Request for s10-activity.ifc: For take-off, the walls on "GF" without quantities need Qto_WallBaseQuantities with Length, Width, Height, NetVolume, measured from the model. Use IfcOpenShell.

First a look at what the model holds.

```python
import ifcopenshell
import ifcopenshell.util.element
import ifcopenshell.util.unit

model = ifcopenshell.open("s10-activity.ifc")
print(model.schema)
for unit_type in ("LENGTHUNIT", "AREAUNIT", "VOLUMEUNIT"):
    print(unit_type, ifcopenshell.util.unit.calculate_unit_scale(model, unit_type))
storey = next(s for s in model.by_type("IfcBuildingStorey") if s.Name == "GF")
walls = [e for e in ifcopenshell.util.element.get_decomposition(storey) if e.is_a("IfcWall")]
for e in sorted(walls, key=lambda e: e.id()):
    print(e.id(), e.is_a(), e.Name, list(ifcopenshell.util.element.get_psets(e, qtos_only=True)), sep=" | ")
```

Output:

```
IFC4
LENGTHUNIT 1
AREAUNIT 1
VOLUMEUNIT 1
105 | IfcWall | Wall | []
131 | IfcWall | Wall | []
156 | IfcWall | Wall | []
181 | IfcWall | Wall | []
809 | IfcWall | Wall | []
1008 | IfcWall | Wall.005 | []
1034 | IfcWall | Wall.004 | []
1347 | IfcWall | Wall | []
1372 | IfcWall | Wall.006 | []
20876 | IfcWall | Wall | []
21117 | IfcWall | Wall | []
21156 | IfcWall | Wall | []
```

```python
import ifcopenshell
import ifcopenshell.api.pset
import ifcopenshell.geom
import ifcopenshell.util.element
import ifcopenshell.util.shape
import ifcopenshell.util.unit

model = ifcopenshell.open("s10-activity.ifc")
unit_scale = ifcopenshell.util.unit.calculate_unit_scale(model)
volume_scale = ifcopenshell.util.unit.calculate_unit_scale(model, "VOLUMEUNIT")
settings = ifcopenshell.geom.settings()

storey = next(s for s in model.by_type("IfcBuildingStorey") if s.Name == "GF")
walls = [e for e in ifcopenshell.util.element.get_decomposition(storey) if e.is_a("IfcWall")]

for e in sorted(walls, key=lambda e: e.id()):
    if ifcopenshell.util.element.get_psets(e, qtos_only=True, should_inherit=False):
        continue
    # Geometry comes back in metres, in the element's own axes.
    shape = ifcopenshell.geom.create_shape(settings, e)
    values = {
        "Length": ifcopenshell.util.shape.get_x(shape.geometry) / unit_scale,
        "Width": ifcopenshell.util.shape.get_y(shape.geometry) / unit_scale,
        "Height": ifcopenshell.util.shape.get_z(shape.geometry) / unit_scale,
        "NetVolume": ifcopenshell.util.shape.get_volume(shape.geometry) / volume_scale,
    }
    qto = ifcopenshell.api.pset.add_qto(model, product=e, name="Qto_WallBaseQuantities")
    ifcopenshell.api.pset.edit_qto(model, qto=qto, properties=values)
    print(e.id(), {k: round(v, 3) for k, v in values.items()})

model.write("s10-activity_rev.ifc")
```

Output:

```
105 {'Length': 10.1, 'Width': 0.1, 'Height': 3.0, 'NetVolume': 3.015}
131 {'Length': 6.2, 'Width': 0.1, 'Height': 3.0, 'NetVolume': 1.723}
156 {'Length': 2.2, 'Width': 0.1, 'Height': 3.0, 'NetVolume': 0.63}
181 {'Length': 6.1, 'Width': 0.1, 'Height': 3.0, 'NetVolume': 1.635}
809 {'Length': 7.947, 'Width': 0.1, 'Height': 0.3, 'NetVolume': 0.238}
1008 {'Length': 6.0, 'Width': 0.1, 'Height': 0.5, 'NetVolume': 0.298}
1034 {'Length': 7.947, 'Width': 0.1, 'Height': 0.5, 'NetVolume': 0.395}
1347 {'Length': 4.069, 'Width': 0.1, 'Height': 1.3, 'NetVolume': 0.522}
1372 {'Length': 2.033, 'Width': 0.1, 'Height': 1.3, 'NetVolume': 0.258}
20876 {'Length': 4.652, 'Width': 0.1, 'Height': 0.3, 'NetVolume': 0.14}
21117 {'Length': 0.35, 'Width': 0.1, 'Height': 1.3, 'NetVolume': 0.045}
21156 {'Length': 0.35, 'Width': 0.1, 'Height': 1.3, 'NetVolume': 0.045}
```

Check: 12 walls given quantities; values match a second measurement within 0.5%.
